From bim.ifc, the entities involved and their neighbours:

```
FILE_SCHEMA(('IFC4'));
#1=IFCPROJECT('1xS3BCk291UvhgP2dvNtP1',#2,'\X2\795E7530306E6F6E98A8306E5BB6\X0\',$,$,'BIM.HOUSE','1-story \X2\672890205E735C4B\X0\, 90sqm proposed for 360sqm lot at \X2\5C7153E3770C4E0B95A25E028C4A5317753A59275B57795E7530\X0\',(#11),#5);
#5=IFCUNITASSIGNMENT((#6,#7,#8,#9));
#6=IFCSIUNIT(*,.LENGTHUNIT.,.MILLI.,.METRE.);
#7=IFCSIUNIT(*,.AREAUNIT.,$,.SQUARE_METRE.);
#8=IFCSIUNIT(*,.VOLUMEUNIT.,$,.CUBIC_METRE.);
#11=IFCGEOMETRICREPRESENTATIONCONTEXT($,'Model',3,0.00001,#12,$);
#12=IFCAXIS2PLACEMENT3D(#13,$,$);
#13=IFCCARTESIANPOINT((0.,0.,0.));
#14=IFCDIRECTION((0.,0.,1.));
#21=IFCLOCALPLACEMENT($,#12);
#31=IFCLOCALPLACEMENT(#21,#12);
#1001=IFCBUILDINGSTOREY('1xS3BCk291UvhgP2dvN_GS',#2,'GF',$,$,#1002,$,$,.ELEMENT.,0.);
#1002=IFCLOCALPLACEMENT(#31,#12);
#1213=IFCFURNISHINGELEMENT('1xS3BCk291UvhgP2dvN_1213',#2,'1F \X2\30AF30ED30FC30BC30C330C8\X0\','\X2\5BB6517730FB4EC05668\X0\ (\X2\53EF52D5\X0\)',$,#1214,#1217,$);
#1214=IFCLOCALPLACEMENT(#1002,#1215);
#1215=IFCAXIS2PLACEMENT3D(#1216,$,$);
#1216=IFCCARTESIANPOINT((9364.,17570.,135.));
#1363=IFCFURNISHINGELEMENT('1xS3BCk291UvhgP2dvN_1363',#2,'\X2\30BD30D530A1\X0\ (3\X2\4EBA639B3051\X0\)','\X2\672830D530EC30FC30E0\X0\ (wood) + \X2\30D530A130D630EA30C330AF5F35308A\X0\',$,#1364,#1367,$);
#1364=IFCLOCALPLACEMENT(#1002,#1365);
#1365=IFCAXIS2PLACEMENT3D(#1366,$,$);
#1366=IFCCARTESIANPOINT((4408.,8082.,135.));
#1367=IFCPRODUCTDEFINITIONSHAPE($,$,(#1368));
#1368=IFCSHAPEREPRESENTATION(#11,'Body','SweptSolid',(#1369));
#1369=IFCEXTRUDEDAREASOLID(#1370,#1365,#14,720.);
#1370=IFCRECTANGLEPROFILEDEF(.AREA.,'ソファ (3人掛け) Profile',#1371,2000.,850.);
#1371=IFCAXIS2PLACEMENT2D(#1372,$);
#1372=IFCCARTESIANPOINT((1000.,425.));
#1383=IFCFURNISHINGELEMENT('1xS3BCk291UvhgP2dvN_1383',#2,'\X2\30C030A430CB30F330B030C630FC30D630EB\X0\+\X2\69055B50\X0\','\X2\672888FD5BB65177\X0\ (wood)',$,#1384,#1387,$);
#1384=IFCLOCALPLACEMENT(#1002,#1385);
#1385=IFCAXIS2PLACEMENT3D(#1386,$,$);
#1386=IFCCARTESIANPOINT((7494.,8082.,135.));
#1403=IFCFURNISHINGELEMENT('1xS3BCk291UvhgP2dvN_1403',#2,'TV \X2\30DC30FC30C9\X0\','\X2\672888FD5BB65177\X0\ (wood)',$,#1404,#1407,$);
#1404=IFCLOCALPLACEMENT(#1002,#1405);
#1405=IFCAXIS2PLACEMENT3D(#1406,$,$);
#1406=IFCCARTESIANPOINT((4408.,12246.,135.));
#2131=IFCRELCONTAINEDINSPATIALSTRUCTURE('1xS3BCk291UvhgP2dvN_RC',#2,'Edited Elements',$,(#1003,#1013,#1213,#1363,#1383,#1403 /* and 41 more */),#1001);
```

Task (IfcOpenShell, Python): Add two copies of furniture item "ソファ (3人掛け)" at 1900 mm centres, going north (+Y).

```python
import numpy as np
import ifcopenshell
import ifcopenshell.api.geometry
import ifcopenshell.api.root
import ifcopenshell.util.element
import ifcopenshell.util.placement

model = ifcopenshell.open("bim.ifc")


def reuse_history(source, copy):
    """copy_class also copies each property set's owner history, people and application; keep the originals."""
    for rel in copy.IsDefinedBy:
        if rel.is_a("IfcRelDefinesByProperties") and (history := rel.RelatingPropertyDefinition.OwnerHistory):
            rel.RelatingPropertyDefinition.OwnerHistory = source.OwnerHistory
            ifcopenshell.util.element.remove_deep2(model, history)


source = model.by_id(1363)
base = ifcopenshell.util.placement.get_local_placement(source.ObjectPlacement)
step = np.array([0.0, 1.0, 0.0]) * 1900.0

for i in range(1, 3):
    copy = ifcopenshell.api.root.copy_class(model, product=source)
    copy.Representation = ifcopenshell.util.element.copy_deep(
        model, source.Representation, exclude=["IfcGeometricRepresentationContext", "IfcRepresentationMap"]
    )
    reuse_history(source, copy)
    matrix = base.copy()
    matrix[:3, 3] += i * step
    print("added at", matrix[:3, 3].round(3) + 0.0)
    ifcopenshell.api.geometry.edit_object_placement(model, product=copy, matrix=matrix, is_si=False)

model.write("bim_updated.ifc")
```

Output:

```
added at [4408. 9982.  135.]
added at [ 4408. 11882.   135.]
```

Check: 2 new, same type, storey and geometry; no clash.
